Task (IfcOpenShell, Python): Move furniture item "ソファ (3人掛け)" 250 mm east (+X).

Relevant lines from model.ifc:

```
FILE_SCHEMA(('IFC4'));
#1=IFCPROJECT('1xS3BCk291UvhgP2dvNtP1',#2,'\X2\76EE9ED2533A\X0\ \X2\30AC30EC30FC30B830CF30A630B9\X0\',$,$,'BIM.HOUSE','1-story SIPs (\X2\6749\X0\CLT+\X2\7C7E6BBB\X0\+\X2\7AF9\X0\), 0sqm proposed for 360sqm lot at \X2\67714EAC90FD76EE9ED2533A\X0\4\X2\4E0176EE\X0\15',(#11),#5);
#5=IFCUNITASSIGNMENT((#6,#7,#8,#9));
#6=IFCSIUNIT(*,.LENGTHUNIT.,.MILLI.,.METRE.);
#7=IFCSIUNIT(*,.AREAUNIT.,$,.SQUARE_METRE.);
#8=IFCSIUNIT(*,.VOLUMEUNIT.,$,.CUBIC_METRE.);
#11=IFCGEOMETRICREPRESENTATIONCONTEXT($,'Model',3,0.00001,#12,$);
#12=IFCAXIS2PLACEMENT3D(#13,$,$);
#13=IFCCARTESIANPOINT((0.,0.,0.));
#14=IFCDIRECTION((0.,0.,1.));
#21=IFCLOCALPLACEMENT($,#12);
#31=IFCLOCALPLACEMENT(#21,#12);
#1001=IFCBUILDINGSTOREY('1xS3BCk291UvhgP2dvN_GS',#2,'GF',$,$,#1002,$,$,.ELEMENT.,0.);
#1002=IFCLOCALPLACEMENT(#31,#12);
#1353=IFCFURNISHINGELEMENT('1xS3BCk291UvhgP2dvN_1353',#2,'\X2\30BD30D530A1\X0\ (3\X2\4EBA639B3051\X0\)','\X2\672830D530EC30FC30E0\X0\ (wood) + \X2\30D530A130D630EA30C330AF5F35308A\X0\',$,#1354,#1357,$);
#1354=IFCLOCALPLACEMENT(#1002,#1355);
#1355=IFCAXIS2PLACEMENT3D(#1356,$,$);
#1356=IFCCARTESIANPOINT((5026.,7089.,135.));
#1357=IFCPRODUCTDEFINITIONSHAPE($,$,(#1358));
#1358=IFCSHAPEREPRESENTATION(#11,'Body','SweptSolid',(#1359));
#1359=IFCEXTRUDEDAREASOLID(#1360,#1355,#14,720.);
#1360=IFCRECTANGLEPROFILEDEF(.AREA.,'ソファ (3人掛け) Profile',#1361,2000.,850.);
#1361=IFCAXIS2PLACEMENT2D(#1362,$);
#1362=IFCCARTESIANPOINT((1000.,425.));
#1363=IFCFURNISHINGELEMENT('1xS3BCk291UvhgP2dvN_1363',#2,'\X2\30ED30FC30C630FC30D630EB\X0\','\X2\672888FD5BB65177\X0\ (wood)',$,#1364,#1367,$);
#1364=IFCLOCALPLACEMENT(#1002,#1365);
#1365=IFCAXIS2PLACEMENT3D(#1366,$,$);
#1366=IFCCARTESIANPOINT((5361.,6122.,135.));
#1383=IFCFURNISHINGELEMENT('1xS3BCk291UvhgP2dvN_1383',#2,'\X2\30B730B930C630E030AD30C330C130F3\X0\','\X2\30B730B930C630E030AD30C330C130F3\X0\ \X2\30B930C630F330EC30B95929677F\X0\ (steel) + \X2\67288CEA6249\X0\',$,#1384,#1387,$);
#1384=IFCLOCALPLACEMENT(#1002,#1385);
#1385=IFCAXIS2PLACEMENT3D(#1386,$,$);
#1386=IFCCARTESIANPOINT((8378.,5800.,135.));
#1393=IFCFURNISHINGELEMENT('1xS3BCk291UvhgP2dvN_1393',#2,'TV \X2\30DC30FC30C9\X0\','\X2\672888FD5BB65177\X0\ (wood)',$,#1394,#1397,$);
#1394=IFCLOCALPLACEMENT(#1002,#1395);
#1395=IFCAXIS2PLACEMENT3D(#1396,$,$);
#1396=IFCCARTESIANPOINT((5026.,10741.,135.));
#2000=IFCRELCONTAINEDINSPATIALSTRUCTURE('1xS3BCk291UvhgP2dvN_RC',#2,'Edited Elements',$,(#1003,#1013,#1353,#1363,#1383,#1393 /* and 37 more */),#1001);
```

```python
import ifcopenshell
import ifcopenshell.api.geometry
import ifcopenshell.util.placement

model = ifcopenshell.open("model.ifc")

item = model.by_id(1353)
matrix = ifcopenshell.util.placement.get_local_placement(item.ObjectPlacement)
matrix[0, 3] += 250.0
ifcopenshell.api.geometry.edit_object_placement(model, product=item, matrix=matrix, is_si=False)

print(ifcopenshell.util.placement.get_local_placement(item.ObjectPlacement).round(3) + 0.0)

model.write("model_rev.ifc")
```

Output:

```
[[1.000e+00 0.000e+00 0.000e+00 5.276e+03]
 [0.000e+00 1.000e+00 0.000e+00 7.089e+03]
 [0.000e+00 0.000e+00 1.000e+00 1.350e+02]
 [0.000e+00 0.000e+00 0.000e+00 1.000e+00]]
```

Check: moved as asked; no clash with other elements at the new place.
